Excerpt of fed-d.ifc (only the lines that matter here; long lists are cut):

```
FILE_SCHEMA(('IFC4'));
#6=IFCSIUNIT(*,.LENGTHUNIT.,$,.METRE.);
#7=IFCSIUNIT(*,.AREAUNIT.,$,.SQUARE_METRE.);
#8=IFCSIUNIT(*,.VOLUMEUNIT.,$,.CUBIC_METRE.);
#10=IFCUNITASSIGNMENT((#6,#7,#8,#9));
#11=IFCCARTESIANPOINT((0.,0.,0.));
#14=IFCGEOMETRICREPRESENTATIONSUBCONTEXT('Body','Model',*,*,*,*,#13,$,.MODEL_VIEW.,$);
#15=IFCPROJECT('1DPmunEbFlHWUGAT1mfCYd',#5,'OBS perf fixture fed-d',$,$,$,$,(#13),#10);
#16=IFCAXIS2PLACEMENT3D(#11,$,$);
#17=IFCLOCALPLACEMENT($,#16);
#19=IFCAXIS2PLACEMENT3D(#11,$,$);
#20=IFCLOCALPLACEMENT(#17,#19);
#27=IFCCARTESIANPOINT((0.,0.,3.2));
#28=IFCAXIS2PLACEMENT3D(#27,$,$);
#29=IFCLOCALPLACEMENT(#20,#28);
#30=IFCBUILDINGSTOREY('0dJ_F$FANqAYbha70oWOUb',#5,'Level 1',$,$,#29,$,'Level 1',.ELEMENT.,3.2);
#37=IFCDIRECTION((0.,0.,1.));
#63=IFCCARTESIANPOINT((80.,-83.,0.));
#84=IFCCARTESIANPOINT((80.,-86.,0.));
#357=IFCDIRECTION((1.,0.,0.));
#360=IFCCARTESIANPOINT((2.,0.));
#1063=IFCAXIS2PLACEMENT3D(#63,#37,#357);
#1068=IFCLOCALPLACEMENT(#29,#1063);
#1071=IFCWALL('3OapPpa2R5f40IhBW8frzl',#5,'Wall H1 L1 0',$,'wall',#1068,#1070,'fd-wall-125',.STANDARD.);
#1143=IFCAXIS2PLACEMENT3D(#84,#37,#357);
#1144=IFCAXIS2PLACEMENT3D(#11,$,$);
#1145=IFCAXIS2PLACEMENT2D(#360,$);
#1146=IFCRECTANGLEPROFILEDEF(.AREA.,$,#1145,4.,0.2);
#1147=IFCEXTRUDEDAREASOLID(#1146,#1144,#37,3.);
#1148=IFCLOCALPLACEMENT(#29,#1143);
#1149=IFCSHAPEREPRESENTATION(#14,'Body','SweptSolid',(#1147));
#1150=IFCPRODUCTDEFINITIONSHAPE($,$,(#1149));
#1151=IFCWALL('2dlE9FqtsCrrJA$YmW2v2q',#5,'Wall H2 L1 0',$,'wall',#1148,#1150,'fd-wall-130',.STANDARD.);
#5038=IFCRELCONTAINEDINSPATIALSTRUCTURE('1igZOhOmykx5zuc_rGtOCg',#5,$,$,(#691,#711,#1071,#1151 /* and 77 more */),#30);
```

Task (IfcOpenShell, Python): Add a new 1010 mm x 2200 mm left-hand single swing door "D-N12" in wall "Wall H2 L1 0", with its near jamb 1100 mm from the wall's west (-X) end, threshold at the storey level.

```python
import numpy as np
import ifcopenshell
import ifcopenshell.api.feature
import ifcopenshell.api.geometry
import ifcopenshell.api.root
import ifcopenshell.api.spatial
import ifcopenshell.geom
import ifcopenshell.util.element
import ifcopenshell.util.placement
import ifcopenshell.util.representation
import ifcopenshell.util.shape
import ifcopenshell.util.unit

model = ifcopenshell.open("fed-d.ifc")
unit_scale = ifcopenshell.util.unit.calculate_unit_scale(model)
settings = ifcopenshell.geom.settings()


def volume(element):
    """Net volume in cubic metres, openings subtracted."""
    shape = ifcopenshell.geom.create_shape(settings, element)
    return ifcopenshell.util.shape.get_volume(shape.geometry)


wall = model.by_id(1151)
storey = ifcopenshell.util.element.get_container(wall, ifc_class="IfcBuildingStorey")
context = ifcopenshell.util.representation.get_context(model, "Model", "Body", "MODEL_VIEW")
before = volume(wall)

width, height, from_end, sill = 1.01, 2.2, 1.1, 0.0  # metres

# The wall runs along its own X axis, and the end named is its -X end.
wall_shape = ifcopenshell.geom.create_shape(settings, wall)
x, y, z = ifcopenshell.util.shape.get_vertices(wall_shape.geometry).T
start = x.min() + from_end
face, thickness = float(y.min()), float(y.max() - y.min())
wall_matrix = ifcopenshell.util.placement.get_local_placement(wall.ObjectPlacement)
level = ifcopenshell.util.placement.get_local_placement(storey.ObjectPlacement)[2, 3]


def in_wall(x, y):
    """Placement at x, y metres in the wall's axes, at sill height."""
    matrix = wall_matrix.copy()
    matrix[:, 3] = wall_matrix @ np.array([x / unit_scale, y / unit_scale, 0.0, 1.0])
    matrix[2, 3] = level + sill / unit_scale
    return matrix


# Opening: a box that overshoots both wall faces by 50 mm.
opening = ifcopenshell.api.root.create_entity(model, ifc_class="IfcOpeningElement", predefined_type="OPENING")
box = ifcopenshell.api.geometry.add_wall_representation(
    model, context=context, length=width, height=height, thickness=thickness + 0.1
)
ifcopenshell.api.geometry.assign_representation(model, product=opening, representation=box)
ifcopenshell.api.geometry.edit_object_placement(model, product=opening, matrix=in_wall(start, face - 0.05), is_si=False)
ifcopenshell.api.feature.add_feature(model, feature=opening, element=wall)

door = ifcopenshell.api.root.create_entity(model, ifc_class="IfcDoor", name="D-N12", predefined_type="DOOR")
door.OverallWidth, door.OverallHeight = width / unit_scale, height / unit_scale
door.OperationType = "SINGLE_SWING_LEFT"
body = ifcopenshell.api.geometry.add_door_representation(
    model,
    context=context,
    overall_width=door.OverallWidth,
    overall_height=door.OverallHeight,
    operation_type="SINGLE_SWING_LEFT",
    lining_properties={"LiningDepth": thickness / unit_scale, "ThresholdDepth": thickness / unit_scale},
)
ifcopenshell.api.geometry.assign_representation(model, product=door, representation=body)
ifcopenshell.api.spatial.assign_container(model, products=[door], relating_structure=storey)
ifcopenshell.api.feature.add_filling(model, opening=opening, element=door)

# The lining spans the wall, so the door starts at the wall face.
ifcopenshell.api.geometry.edit_object_placement(model, product=door, matrix=in_wall(start, face), is_si=False)

after = volume(wall)

print(f"wall volume {before:.3f} -> {after:.3f} m3")

model.write("fed-d_rev.ifc")
```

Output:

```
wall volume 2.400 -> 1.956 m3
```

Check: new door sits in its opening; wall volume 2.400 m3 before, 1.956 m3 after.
